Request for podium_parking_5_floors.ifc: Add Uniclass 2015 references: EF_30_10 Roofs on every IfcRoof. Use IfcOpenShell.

First a look at what the model holds.

```python
import ifcopenshell

model = ifcopenshell.open("podium_parking_5_floors.ifc")
print(model.schema)
print("classifications:", [c.Name for c in model.by_type("IfcClassification")])
for ifc_class in ("IfcDoor", "IfcRoof", "IfcStair", "IfcWall", "IfcWindow"):
    print(ifc_class, len(model.by_type(ifc_class)))
```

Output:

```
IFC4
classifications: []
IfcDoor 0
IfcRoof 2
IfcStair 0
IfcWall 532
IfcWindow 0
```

```python
import ifcopenshell
import ifcopenshell.api.classification

model = ifcopenshell.open("podium_parking_5_floors.ifc")

system = ifcopenshell.api.classification.add_classification(model, classification="Uniclass 2015")

codes = {
    "IfcRoof": ("EF_30_10", "Roofs"),
}
for ifc_class, (code, name) in codes.items():
    products = model.by_type(ifc_class)
    ifcopenshell.api.classification.add_reference(
        model, products=products, classification=system, identification=code, name=name
    )
    print(code, len(products))

model.write("podium_parking_5_floors_v2.ifc")
```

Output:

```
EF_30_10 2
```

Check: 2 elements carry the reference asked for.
